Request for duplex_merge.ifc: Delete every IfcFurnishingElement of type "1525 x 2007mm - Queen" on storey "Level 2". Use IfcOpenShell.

First a look at what the model holds.

```python
import ifcopenshell
import ifcopenshell.util.element

model = ifcopenshell.open("duplex_merge.ifc")
print(model.schema)
storey = next(s for s in model.by_type("IfcBuildingStorey") if s.Name == "Level 2")
furniture = [e for e in ifcopenshell.util.element.get_decomposition(storey) if e.is_a("IfcFurnishingElement")]
seen = {}
for e in furniture:
    element_type = ifcopenshell.util.element.get_type(e)
    name = element_type.Name if element_type not in (None, e) else None
    seen[name] = seen.get(name, 0) + 1
for name, count in sorted(seen.items(), key=str):
    print(count, "x", name)
```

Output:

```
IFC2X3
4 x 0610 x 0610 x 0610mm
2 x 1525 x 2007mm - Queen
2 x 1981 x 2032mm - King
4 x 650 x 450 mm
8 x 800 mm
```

```python
import ifcopenshell
import ifcopenshell.api.root
import ifcopenshell.util.element

model = ifcopenshell.open("duplex_merge.ifc")

storey = next(s for s in model.by_type("IfcBuildingStorey") if s.Name == "Level 2")
furniture = [e for e in ifcopenshell.util.element.get_decomposition(storey) if e.is_a("IfcFurnishingElement")]
targets = [e for e in furniture if (t := ifcopenshell.util.element.get_type(e)) not in (None, e) and t.Name == "1525 x 2007mm - Queen"]

for e in targets:
    ifcopenshell.api.root.remove_product(model, product=e)
print(len(targets), "removed")

model.write("duplex_merge-out.ifc")
```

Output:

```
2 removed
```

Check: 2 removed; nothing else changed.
